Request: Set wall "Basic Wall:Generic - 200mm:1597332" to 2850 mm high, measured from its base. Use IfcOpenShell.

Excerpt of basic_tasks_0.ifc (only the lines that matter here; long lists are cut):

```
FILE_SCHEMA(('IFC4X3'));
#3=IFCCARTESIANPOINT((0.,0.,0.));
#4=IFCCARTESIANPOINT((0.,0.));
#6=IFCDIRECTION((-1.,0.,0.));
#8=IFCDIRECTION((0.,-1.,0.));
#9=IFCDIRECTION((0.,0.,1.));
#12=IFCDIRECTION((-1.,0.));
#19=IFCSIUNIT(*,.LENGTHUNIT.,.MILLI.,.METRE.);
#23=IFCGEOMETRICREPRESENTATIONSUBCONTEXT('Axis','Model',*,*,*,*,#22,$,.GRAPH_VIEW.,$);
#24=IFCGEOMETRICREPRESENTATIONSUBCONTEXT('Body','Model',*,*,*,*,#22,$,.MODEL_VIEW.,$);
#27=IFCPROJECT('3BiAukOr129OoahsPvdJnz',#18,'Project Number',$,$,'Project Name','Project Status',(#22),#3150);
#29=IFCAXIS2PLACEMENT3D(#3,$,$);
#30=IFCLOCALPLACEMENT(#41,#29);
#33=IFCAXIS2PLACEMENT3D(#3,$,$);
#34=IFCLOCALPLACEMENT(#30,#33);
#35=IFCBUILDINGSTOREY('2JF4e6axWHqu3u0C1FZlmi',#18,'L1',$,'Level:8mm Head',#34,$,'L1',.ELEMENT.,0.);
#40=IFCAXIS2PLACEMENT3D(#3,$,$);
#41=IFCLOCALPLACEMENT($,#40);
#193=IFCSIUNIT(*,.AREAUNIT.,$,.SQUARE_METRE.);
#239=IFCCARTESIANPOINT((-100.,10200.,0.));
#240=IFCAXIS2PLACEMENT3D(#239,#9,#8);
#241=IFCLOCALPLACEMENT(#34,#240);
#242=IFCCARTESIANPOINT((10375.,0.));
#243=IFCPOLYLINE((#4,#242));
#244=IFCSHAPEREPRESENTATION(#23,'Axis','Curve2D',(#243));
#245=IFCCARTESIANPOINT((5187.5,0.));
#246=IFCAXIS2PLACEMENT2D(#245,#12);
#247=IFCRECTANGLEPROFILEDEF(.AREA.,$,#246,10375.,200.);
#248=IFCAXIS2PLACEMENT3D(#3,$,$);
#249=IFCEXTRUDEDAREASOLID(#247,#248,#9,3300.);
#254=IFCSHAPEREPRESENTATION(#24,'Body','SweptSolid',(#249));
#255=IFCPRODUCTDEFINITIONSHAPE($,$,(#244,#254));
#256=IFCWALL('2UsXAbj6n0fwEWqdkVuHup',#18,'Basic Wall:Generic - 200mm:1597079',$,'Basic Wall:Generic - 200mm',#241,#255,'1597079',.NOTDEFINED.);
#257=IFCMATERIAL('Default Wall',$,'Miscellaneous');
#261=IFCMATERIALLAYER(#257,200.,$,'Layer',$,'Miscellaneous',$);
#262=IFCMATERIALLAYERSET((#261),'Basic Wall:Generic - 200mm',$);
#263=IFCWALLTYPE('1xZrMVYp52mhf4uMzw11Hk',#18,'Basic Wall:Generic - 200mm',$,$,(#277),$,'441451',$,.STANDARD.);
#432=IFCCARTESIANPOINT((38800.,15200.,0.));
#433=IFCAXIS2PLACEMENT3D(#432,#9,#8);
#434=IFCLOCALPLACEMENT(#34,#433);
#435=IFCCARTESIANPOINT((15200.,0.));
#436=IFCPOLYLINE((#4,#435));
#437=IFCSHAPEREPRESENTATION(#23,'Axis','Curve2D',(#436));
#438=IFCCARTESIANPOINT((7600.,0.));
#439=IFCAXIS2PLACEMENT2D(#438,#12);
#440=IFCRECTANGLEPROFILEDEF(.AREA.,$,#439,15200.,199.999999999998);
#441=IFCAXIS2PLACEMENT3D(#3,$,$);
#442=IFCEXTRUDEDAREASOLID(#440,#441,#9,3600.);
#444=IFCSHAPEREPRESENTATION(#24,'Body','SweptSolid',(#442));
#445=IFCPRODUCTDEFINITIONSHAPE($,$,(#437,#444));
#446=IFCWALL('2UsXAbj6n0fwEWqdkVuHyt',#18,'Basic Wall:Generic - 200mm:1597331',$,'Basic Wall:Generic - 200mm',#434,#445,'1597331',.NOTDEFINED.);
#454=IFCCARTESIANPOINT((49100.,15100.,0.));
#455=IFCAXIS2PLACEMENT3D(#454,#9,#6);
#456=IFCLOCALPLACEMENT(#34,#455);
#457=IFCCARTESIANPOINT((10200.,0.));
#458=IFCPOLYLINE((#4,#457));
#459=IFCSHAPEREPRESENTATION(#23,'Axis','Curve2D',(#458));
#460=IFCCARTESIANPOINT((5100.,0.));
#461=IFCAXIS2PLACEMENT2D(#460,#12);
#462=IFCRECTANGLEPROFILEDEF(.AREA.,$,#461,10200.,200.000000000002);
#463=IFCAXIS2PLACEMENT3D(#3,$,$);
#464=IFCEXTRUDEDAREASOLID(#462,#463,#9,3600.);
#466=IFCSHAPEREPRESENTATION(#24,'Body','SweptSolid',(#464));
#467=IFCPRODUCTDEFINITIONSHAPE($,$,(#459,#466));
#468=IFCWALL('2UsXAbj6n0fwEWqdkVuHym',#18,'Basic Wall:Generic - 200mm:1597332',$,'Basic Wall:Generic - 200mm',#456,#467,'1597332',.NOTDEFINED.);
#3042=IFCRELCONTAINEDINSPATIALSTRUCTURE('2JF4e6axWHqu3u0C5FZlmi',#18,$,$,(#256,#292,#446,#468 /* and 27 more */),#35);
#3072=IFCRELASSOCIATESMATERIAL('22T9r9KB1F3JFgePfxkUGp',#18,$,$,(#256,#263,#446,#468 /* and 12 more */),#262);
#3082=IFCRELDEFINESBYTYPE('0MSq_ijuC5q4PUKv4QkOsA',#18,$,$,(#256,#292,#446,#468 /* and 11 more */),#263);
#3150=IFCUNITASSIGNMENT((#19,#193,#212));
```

```python
import ifcopenshell
import ifcopenshell.geom
import ifcopenshell.util.representation
import ifcopenshell.util.shape

model = ifcopenshell.open("basic_tasks_0.ifc")
settings = ifcopenshell.geom.settings()


def volume(element):
    """Net volume in cubic metres, openings subtracted."""
    shape = ifcopenshell.geom.create_shape(settings, element)
    return ifcopenshell.util.shape.get_volume(shape.geometry)


wall = model.by_id(468)
before = volume(wall)

body = ifcopenshell.util.representation.get_representation(wall, "Model", "Body")
solid = body.Items[0]
old_height = solid.Depth
solid.Depth = 2850.0
after = volume(wall)

print(f"height {old_height:g} -> {solid.Depth:g}, volume {before:.3f} -> {after:.3f} m3")

model.write("basic_tasks_0_edited.ifc")
```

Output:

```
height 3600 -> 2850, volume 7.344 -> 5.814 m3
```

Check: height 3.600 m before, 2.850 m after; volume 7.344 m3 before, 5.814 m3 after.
